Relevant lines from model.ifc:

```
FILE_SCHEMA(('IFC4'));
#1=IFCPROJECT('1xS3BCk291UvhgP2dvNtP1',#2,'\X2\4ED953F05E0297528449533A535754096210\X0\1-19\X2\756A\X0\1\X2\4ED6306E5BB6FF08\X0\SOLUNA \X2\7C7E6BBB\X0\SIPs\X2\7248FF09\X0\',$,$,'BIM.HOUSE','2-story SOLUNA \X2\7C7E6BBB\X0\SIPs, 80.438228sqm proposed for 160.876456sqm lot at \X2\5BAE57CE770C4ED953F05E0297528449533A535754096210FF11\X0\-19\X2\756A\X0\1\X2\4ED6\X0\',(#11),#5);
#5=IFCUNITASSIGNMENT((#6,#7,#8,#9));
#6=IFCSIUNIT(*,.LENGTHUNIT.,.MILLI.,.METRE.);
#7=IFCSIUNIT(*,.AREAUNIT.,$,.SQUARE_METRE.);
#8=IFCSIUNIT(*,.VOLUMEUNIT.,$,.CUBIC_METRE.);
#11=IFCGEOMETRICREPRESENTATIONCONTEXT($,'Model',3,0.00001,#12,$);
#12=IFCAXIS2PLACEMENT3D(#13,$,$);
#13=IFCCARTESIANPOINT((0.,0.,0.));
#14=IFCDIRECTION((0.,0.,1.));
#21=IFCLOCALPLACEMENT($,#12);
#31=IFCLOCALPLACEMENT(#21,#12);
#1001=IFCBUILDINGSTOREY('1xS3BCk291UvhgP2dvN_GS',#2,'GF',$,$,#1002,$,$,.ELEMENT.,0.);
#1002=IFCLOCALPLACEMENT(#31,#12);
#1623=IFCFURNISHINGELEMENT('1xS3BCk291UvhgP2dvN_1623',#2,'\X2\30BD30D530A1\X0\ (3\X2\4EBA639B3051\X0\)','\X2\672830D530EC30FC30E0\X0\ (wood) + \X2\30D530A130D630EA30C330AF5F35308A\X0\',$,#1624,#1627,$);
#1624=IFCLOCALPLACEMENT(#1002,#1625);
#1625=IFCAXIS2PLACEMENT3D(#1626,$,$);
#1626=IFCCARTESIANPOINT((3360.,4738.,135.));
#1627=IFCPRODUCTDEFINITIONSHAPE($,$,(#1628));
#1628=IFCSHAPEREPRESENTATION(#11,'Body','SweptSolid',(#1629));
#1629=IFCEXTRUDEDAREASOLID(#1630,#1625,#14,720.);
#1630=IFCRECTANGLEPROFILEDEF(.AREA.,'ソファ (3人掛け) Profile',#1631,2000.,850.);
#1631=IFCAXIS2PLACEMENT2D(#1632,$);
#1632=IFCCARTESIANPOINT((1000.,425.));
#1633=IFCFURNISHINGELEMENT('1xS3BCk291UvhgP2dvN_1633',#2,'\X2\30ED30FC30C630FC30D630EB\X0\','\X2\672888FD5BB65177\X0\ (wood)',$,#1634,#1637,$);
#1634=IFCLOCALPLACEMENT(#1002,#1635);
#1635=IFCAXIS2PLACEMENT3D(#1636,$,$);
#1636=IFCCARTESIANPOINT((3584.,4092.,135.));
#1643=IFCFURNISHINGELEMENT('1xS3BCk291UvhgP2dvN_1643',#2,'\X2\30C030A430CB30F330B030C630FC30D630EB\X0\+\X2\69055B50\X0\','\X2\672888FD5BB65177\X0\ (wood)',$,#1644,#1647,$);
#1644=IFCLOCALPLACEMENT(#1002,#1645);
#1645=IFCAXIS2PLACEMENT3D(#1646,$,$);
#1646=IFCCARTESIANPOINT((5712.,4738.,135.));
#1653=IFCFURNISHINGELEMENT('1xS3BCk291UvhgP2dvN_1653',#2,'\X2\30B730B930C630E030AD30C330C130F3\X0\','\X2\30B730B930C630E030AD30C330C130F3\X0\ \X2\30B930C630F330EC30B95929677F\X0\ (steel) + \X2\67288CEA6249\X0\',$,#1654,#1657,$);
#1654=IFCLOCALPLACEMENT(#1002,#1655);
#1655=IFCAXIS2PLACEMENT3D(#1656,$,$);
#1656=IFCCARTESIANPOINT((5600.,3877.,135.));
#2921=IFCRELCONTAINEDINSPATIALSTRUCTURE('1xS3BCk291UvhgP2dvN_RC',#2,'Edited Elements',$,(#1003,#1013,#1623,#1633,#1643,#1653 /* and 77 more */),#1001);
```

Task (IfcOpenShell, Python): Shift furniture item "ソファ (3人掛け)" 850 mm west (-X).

```python
import ifcopenshell
import ifcopenshell.api.geometry
import ifcopenshell.util.placement

model = ifcopenshell.open("model.ifc")

item = model.by_guid("1xS3BCk291UvhgP2dvN_1623")
matrix = ifcopenshell.util.placement.get_local_placement(item.ObjectPlacement)
matrix[0, 3] -= 850.0
ifcopenshell.api.geometry.edit_object_placement(model, product=item, matrix=matrix, is_si=False)

print(ifcopenshell.util.placement.get_local_placement(item.ObjectPlacement).round(3) + 0.0)

model.write("model_edited.ifc")
```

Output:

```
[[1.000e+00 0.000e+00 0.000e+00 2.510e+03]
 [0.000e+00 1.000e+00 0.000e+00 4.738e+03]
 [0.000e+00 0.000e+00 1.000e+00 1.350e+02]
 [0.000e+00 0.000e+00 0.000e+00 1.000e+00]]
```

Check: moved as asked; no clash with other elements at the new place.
